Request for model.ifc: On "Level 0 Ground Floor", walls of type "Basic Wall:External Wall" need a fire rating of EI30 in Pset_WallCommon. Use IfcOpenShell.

First a look at what the model holds.

```python
import ifcopenshell
import ifcopenshell.util.element

model = ifcopenshell.open("model.ifc")
print(model.schema)
storey = next(s for s in model.by_type("IfcBuildingStorey") if s.Name == "Level 0 Ground Floor")
walls = [e for e in ifcopenshell.util.element.get_decomposition(storey) if e.is_a("IfcWall")]
seen = {}
for e in walls:
    element_type = ifcopenshell.util.element.get_type(e)
    key = (element_type.Name if element_type != e and element_type else None, ifcopenshell.util.element.get_pset(e, "Pset_WallCommon", "FireRating"))
    seen[key] = seen.get(key, 0) + 1
for (name, value), count in sorted(seen.items(), key=str):
    print(count, "x", name, "|", value)
```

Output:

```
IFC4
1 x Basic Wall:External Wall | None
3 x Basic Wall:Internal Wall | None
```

```python
import ifcopenshell
import ifcopenshell.api.pset
import ifcopenshell.util.element

model = ifcopenshell.open("model.ifc")

storey = next(s for s in model.by_type("IfcBuildingStorey") if s.Name == "Level 0 Ground Floor")
walls = [e for e in ifcopenshell.util.element.get_decomposition(storey) if e.is_a("IfcWall")]

count = 0
for e in walls:
    element_type = ifcopenshell.util.element.get_type(e)
    if element_type in (None, e) or element_type.Name != "Basic Wall:External Wall":
        continue
    # add_pset returns the element's existing set when there is one.
    pset = ifcopenshell.api.pset.add_pset(model, product=e, name="Pset_WallCommon")
    ifcopenshell.api.pset.edit_pset(model, pset=pset, properties={"FireRating": "EI30"})
    count += 1

print(count, "walls updated")

model.write("model_v2.ifc")
```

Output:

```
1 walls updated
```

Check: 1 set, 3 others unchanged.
